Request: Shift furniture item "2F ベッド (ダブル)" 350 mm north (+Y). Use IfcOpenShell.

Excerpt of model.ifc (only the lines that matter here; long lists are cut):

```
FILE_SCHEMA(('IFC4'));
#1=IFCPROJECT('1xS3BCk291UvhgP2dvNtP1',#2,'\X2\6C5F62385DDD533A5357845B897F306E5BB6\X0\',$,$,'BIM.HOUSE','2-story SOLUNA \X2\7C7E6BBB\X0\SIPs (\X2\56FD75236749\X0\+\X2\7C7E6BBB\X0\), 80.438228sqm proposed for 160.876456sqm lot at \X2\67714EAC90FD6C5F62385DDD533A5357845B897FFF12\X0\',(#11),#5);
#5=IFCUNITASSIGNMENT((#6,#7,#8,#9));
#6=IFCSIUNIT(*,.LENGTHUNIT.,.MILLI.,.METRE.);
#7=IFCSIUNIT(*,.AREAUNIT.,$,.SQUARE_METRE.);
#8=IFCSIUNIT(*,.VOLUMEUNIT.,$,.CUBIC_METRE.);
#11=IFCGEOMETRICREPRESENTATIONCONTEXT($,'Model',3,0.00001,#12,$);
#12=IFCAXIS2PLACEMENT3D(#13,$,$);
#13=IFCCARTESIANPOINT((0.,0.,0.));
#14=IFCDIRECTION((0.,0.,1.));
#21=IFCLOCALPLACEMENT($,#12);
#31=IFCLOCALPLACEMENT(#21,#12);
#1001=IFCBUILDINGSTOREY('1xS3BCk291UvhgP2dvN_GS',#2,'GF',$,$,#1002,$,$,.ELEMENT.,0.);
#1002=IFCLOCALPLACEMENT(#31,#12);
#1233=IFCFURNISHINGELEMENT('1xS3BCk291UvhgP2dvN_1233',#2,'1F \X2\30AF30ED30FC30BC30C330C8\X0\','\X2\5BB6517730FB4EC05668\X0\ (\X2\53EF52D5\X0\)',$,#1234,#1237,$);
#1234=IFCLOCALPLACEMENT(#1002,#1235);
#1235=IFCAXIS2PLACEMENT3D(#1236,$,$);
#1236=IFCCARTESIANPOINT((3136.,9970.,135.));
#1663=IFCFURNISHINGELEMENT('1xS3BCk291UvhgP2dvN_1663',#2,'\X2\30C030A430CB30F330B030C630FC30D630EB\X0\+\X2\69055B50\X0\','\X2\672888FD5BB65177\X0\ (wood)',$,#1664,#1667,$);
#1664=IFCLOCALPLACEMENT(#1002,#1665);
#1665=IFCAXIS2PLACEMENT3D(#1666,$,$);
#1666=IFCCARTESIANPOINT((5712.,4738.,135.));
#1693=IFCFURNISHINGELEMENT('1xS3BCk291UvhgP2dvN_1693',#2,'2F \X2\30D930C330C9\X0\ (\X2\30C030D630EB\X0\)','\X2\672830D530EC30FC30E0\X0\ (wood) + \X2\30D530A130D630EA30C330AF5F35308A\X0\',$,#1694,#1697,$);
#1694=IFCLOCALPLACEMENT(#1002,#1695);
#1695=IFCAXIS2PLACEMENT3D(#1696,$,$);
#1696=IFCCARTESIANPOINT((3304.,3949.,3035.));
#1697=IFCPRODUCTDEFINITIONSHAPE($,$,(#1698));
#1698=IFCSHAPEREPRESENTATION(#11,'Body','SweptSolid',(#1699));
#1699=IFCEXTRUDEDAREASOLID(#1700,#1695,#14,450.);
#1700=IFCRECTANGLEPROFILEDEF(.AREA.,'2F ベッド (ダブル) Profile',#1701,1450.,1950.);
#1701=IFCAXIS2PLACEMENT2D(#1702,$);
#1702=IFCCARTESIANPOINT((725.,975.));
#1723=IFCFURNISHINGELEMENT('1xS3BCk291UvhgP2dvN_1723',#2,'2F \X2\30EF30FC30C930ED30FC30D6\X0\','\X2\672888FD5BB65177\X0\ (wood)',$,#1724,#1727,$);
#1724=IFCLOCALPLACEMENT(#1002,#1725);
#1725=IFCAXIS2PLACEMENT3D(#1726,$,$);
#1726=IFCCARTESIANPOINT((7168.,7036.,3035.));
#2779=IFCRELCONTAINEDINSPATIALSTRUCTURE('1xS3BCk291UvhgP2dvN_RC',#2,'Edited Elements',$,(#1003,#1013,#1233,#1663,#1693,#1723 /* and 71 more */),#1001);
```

```python
import ifcopenshell
import ifcopenshell.api.geometry
import ifcopenshell.util.placement
import ifcopenshell.util.unit

model = ifcopenshell.open("model.ifc")
unit_scale = ifcopenshell.util.unit.calculate_unit_scale(model)

item = model.by_id(1693)
matrix = ifcopenshell.util.placement.get_local_placement(item.ObjectPlacement)
matrix[1, 3] += 0.35 / unit_scale
ifcopenshell.api.geometry.edit_object_placement(model, product=item, matrix=matrix, is_si=False)

print(ifcopenshell.util.placement.get_local_placement(item.ObjectPlacement).round(3) + 0.0)

model.write("model_rev.ifc")
```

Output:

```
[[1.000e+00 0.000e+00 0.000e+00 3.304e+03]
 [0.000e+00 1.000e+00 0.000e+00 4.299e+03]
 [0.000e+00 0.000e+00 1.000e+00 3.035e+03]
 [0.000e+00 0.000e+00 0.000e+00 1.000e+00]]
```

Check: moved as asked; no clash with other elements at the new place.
